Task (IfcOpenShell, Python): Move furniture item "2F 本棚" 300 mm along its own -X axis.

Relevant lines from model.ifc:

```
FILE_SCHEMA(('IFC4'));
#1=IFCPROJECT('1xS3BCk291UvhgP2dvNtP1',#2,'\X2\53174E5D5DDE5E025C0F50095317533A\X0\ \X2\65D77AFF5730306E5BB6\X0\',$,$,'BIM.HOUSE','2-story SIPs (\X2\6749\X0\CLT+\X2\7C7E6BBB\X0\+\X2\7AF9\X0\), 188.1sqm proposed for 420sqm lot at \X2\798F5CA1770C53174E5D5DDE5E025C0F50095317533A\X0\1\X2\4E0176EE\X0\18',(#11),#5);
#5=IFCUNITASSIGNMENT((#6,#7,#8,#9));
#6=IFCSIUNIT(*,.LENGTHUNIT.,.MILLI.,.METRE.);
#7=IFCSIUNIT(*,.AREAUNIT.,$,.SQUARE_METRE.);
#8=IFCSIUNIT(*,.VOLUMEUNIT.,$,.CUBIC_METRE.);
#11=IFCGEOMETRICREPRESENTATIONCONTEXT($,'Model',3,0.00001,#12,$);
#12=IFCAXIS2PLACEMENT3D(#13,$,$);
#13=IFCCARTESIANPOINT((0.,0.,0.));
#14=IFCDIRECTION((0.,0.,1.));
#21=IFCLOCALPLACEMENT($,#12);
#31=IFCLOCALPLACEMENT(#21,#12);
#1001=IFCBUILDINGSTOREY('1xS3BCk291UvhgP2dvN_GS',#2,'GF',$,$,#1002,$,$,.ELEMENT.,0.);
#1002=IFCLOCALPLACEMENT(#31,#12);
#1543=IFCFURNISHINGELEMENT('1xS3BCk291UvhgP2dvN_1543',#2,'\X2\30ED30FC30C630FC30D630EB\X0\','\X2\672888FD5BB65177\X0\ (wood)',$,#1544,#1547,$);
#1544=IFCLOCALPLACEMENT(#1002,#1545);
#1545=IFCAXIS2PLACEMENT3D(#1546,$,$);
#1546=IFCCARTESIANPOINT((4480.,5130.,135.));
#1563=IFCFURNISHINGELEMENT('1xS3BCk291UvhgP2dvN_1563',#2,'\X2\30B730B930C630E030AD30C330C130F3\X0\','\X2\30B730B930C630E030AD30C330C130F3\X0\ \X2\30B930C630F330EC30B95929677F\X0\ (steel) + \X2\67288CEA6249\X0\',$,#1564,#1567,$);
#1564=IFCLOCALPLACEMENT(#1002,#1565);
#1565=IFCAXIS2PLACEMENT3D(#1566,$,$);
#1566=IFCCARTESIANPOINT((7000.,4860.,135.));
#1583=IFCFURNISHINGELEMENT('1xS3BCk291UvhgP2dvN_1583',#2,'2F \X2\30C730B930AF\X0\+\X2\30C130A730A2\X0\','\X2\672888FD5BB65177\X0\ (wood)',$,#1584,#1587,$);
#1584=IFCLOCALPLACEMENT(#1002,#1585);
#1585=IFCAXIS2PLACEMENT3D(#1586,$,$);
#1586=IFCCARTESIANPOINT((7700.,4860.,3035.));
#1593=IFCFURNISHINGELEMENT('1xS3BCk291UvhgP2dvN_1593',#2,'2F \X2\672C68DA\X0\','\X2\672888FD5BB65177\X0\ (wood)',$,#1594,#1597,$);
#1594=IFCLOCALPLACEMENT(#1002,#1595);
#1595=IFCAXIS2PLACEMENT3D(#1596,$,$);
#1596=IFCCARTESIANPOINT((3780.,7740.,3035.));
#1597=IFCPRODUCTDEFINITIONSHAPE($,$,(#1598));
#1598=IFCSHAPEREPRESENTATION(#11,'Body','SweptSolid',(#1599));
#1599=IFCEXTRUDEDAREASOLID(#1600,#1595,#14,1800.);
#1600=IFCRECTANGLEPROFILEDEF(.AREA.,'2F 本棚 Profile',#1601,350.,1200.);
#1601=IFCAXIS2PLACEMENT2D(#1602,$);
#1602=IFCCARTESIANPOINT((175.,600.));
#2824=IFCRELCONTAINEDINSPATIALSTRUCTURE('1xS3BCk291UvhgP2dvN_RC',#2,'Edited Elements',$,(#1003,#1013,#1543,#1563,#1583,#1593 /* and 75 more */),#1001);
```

```python
import ifcopenshell
import ifcopenshell.api.geometry
import ifcopenshell.util.placement

model = ifcopenshell.open("model.ifc")

item = model.by_id(1593)
matrix = ifcopenshell.util.placement.get_local_placement(item.ObjectPlacement)
matrix[:3, 3] -= matrix[:3, 0] * 300.0
ifcopenshell.api.geometry.edit_object_placement(model, product=item, matrix=matrix, is_si=False)

print(ifcopenshell.util.placement.get_local_placement(item.ObjectPlacement).round(3) + 0.0)

model.write("model_v2.ifc")
```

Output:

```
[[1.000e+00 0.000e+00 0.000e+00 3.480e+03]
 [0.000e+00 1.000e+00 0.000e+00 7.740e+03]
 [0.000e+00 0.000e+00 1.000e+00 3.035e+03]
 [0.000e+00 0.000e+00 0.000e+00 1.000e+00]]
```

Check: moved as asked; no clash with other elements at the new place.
